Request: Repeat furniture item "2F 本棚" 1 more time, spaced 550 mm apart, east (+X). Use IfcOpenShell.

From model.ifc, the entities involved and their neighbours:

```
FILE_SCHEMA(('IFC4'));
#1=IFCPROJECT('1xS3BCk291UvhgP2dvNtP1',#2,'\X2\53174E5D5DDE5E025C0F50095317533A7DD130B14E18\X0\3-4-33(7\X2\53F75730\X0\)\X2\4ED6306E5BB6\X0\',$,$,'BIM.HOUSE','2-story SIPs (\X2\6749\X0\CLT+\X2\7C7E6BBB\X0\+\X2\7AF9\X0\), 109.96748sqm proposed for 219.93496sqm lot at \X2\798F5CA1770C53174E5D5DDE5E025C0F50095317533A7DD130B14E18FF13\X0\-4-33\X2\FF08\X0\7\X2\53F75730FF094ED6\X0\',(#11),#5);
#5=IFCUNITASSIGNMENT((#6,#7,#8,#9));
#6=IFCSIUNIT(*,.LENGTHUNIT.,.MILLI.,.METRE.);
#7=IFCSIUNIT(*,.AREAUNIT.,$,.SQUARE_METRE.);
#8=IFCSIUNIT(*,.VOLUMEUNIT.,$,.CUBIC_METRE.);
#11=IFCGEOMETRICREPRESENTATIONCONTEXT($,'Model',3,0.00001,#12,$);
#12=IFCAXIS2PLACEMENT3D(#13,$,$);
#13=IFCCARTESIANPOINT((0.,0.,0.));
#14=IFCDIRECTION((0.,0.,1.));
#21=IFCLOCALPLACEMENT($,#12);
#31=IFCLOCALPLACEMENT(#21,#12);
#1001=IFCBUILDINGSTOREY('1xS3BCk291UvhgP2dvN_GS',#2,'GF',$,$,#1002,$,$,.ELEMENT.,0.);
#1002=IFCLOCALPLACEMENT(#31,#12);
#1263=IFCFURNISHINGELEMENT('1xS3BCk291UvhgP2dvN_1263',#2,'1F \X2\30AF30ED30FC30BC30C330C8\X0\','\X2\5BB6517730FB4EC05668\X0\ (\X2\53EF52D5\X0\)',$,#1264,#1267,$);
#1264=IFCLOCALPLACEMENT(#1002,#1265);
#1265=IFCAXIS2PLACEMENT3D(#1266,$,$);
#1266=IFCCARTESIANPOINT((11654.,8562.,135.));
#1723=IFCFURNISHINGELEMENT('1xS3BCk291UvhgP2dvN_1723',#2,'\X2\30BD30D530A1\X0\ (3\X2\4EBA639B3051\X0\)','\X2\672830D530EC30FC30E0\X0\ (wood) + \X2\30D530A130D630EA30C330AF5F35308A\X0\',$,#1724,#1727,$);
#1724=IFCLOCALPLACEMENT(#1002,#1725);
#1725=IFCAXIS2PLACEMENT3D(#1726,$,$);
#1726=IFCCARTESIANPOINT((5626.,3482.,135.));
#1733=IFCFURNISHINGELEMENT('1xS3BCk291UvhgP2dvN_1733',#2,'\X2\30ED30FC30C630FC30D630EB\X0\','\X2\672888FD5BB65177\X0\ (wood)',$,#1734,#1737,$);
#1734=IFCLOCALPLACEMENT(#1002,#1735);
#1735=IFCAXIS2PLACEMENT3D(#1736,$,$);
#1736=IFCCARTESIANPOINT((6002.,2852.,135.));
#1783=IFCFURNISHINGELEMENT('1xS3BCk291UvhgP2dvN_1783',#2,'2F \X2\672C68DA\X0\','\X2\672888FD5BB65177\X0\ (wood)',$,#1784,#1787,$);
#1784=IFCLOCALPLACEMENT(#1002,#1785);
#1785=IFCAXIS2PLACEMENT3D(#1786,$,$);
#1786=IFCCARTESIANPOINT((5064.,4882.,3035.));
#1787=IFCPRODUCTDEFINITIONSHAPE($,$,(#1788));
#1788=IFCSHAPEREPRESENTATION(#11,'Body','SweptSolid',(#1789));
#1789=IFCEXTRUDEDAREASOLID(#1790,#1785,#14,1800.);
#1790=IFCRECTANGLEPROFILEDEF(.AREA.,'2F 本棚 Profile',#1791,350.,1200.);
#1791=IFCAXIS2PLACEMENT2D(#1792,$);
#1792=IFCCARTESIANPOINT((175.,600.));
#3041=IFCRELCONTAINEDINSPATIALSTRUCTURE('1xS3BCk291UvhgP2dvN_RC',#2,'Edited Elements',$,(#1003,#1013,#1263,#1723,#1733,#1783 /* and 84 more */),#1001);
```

```python
import numpy as np
import ifcopenshell
import ifcopenshell.api.geometry
import ifcopenshell.api.root
import ifcopenshell.util.element
import ifcopenshell.util.placement
import ifcopenshell.util.unit

model = ifcopenshell.open("model.ifc")
unit_scale = ifcopenshell.util.unit.calculate_unit_scale(model)


def reuse_history(source, copy):
    """copy_class also copies each property set's owner history, people and application; keep the originals."""
    for rel in copy.IsDefinedBy:
        if rel.is_a("IfcRelDefinesByProperties") and (history := rel.RelatingPropertyDefinition.OwnerHistory):
            rel.RelatingPropertyDefinition.OwnerHistory = source.OwnerHistory
            ifcopenshell.util.element.remove_deep2(model, history)


source = model.by_guid("1xS3BCk291UvhgP2dvN_1783")
base = ifcopenshell.util.placement.get_local_placement(source.ObjectPlacement)
step = np.array([1.0, 0.0, 0.0]) * 0.55 / unit_scale

for i in range(1, 2):
    copy = ifcopenshell.api.root.copy_class(model, product=source)
    copy.Representation = ifcopenshell.util.element.copy_deep(
        model, source.Representation, exclude=["IfcGeometricRepresentationContext", "IfcRepresentationMap"]
    )
    reuse_history(source, copy)
    matrix = base.copy()
    matrix[:3, 3] += i * step
    print("added at", matrix[:3, 3].round(3) + 0.0)
    ifcopenshell.api.geometry.edit_object_placement(model, product=copy, matrix=matrix, is_si=False)

model.write("model_rev.ifc")
```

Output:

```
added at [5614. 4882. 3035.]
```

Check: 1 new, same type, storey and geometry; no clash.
